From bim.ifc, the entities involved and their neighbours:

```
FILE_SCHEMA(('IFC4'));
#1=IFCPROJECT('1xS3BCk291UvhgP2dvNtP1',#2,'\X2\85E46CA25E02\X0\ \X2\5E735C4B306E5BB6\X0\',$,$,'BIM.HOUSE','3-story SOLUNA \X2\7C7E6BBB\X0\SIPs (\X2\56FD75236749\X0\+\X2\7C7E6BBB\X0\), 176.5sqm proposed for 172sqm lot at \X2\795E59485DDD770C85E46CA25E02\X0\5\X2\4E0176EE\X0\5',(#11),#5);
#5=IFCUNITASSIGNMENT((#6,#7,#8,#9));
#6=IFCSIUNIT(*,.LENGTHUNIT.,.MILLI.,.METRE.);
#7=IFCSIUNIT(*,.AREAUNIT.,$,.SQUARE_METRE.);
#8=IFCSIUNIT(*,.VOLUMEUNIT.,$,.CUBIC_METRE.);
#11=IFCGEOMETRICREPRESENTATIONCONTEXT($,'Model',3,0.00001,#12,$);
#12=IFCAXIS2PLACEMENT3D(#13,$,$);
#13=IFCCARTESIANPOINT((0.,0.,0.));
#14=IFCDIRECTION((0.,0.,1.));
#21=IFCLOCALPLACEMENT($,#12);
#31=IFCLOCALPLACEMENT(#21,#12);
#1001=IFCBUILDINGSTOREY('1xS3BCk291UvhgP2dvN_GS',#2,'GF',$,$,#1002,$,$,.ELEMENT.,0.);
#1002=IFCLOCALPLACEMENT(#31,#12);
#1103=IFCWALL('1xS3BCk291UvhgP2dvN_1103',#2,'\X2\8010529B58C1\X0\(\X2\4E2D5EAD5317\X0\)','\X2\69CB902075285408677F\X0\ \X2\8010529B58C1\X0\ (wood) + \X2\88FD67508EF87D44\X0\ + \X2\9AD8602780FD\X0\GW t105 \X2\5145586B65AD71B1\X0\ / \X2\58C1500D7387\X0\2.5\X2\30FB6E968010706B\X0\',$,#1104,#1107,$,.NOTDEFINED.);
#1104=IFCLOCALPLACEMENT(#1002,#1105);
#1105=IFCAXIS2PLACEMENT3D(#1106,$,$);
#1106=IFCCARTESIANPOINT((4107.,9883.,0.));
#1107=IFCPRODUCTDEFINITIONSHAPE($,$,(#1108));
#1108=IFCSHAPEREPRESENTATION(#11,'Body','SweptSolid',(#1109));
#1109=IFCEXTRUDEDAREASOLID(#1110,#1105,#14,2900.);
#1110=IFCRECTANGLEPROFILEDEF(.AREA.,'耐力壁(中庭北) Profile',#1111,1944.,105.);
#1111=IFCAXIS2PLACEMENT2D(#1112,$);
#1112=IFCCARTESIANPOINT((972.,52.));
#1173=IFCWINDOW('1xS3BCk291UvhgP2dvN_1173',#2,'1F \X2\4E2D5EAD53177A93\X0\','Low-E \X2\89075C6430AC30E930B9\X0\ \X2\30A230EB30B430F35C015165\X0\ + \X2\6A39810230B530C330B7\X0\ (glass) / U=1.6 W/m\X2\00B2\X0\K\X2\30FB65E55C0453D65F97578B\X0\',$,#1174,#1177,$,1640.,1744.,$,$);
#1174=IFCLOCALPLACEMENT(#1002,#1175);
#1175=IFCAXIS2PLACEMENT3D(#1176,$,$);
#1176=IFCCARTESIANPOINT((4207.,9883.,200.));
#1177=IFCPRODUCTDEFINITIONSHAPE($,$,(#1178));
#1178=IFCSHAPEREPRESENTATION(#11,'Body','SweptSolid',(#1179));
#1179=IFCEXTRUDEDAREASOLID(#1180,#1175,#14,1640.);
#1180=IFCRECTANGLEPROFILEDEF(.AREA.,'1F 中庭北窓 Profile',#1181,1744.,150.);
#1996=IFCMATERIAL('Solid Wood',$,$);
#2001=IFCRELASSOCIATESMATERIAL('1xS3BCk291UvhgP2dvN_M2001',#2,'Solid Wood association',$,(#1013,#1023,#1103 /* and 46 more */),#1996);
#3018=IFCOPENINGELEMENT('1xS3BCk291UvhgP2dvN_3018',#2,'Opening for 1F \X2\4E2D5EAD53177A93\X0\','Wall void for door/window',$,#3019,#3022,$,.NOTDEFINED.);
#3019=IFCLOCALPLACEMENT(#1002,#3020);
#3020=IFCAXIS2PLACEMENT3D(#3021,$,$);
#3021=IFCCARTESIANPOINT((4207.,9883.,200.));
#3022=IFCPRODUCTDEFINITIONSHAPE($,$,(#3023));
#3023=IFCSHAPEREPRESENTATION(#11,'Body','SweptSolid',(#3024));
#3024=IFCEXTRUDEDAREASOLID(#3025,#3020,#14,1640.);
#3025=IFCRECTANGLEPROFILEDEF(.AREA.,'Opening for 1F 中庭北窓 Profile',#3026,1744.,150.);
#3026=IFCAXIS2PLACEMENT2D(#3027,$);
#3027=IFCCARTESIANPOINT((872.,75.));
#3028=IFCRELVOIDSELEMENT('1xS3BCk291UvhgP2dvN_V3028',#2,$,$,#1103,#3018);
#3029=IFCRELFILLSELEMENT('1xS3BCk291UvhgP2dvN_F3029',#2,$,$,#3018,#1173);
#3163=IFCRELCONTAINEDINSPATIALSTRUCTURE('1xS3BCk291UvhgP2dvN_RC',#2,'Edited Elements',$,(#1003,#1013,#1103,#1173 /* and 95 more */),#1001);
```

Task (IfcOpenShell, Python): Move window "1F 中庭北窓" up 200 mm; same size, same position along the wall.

```python
import numpy as np
import ifcopenshell
import ifcopenshell.api.geometry
import ifcopenshell.util.placement
import ifcopenshell.util.unit

model = ifcopenshell.open("bim.ifc")
unit_scale = ifcopenshell.util.unit.calculate_unit_scale(model)

window = model.by_guid("1xS3BCk291UvhgP2dvN_1173")
opening = window.FillsVoids[0].RelatingOpeningElement
dz = 200.0

shift = np.array([0.0, 0.0, dz])
# The window is not placed relative to its opening, so move both.
for product in (opening, window):
    matrix = ifcopenshell.util.placement.get_local_placement(product.ObjectPlacement)
    matrix[:3, 3] += shift
    ifcopenshell.api.geometry.edit_object_placement(model, product=product, matrix=matrix, is_si=False)

print(f"moved by {dz * unit_scale:+.3f} m")

model.write("bim_rev.ifc")
```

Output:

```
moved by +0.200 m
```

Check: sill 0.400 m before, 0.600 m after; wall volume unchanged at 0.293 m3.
